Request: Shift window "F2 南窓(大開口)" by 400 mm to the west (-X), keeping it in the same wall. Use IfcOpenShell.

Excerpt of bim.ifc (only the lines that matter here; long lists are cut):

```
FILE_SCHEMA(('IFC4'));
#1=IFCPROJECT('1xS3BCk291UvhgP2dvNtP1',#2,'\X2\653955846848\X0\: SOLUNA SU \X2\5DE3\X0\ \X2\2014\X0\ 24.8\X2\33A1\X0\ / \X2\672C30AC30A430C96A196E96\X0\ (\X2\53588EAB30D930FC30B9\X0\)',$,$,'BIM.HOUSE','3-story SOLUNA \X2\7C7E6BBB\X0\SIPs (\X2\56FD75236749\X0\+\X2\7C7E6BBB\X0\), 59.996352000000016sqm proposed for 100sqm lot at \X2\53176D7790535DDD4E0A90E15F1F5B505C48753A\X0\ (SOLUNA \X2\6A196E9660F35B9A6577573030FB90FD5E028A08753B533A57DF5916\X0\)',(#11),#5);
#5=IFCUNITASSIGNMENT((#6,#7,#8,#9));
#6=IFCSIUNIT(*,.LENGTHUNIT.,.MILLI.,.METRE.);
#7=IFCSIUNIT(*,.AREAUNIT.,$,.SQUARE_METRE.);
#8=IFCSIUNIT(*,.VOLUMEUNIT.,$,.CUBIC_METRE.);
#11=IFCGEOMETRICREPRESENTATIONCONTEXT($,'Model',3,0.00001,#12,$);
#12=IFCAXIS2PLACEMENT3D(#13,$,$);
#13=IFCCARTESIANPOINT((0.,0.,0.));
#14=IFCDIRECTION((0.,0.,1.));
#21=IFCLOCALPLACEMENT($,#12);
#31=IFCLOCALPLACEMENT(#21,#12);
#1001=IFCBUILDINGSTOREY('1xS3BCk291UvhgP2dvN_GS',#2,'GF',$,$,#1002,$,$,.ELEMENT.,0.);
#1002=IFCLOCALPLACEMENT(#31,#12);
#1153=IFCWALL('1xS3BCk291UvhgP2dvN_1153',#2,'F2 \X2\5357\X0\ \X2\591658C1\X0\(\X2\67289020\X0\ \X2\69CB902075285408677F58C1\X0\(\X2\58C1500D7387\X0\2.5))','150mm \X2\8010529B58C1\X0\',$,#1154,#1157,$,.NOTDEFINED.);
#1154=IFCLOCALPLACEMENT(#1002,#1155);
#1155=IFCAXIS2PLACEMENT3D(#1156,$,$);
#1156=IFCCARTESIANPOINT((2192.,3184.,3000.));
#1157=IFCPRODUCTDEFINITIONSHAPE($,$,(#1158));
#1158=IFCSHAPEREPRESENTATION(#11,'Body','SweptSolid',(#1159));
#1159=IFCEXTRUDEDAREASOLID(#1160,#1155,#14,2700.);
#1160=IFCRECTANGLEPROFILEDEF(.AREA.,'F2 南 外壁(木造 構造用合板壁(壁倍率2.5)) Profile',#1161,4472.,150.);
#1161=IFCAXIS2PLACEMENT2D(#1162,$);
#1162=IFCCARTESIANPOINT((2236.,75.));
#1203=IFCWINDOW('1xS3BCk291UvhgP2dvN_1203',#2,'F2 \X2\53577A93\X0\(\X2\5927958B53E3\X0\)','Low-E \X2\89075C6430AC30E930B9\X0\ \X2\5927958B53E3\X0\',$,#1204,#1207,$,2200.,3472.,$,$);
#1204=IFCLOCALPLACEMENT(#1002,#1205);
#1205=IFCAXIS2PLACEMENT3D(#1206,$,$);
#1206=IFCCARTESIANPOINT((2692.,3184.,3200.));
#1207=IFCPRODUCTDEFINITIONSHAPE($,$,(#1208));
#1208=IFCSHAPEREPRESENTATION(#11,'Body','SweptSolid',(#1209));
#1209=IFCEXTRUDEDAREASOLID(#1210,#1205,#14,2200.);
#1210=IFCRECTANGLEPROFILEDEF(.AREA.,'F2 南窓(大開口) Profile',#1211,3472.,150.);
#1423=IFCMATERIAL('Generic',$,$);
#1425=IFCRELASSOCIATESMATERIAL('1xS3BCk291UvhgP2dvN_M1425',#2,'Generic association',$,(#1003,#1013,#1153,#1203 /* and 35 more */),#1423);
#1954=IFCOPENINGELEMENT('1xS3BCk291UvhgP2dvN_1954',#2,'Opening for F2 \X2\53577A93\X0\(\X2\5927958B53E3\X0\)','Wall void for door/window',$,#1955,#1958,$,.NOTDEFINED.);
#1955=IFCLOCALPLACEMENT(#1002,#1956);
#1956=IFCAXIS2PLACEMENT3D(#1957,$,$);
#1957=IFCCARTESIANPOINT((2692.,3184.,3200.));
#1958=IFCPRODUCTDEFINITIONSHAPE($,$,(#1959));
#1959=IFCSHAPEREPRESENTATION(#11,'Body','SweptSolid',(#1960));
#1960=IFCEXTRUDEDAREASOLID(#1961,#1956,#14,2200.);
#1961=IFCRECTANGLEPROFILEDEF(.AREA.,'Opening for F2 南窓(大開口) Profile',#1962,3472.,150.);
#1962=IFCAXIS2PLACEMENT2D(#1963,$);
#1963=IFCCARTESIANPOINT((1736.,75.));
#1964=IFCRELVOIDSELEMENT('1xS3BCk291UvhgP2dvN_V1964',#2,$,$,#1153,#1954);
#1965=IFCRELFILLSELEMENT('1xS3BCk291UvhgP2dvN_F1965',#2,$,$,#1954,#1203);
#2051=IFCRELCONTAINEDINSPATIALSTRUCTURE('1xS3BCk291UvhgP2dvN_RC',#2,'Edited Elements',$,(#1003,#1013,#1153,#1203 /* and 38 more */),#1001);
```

```python
import ifcopenshell
import ifcopenshell.api.geometry
import ifcopenshell.util.placement

model = ifcopenshell.open("bim.ifc")

window = model.by_guid("1xS3BCk291UvhgP2dvN_1203")
opening = window.FillsVoids[0].RelatingOpeningElement
wall = opening.VoidsElements[0].RelatingBuildingElement

wall_matrix = ifcopenshell.util.placement.get_local_placement(wall.ObjectPlacement)
shift = wall_matrix[:3, 0] * -400.0
before = ifcopenshell.util.placement.get_local_placement(window.ObjectPlacement)[:3, 3].copy()

# The window is not placed relative to its opening, so move both.
for product in (opening, window):
    matrix = ifcopenshell.util.placement.get_local_placement(product.ObjectPlacement)
    matrix[:3, 3] += shift
    ifcopenshell.api.geometry.edit_object_placement(model, product=product, matrix=matrix, is_si=False)

after = ifcopenshell.util.placement.get_local_placement(window.ObjectPlacement)[:3, 3]
print("window moved by", (after - before).round(3) + 0.0)

model.write("bim_edited.ifc")
```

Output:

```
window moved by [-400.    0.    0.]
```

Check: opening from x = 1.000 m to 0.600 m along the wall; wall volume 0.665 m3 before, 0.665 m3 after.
